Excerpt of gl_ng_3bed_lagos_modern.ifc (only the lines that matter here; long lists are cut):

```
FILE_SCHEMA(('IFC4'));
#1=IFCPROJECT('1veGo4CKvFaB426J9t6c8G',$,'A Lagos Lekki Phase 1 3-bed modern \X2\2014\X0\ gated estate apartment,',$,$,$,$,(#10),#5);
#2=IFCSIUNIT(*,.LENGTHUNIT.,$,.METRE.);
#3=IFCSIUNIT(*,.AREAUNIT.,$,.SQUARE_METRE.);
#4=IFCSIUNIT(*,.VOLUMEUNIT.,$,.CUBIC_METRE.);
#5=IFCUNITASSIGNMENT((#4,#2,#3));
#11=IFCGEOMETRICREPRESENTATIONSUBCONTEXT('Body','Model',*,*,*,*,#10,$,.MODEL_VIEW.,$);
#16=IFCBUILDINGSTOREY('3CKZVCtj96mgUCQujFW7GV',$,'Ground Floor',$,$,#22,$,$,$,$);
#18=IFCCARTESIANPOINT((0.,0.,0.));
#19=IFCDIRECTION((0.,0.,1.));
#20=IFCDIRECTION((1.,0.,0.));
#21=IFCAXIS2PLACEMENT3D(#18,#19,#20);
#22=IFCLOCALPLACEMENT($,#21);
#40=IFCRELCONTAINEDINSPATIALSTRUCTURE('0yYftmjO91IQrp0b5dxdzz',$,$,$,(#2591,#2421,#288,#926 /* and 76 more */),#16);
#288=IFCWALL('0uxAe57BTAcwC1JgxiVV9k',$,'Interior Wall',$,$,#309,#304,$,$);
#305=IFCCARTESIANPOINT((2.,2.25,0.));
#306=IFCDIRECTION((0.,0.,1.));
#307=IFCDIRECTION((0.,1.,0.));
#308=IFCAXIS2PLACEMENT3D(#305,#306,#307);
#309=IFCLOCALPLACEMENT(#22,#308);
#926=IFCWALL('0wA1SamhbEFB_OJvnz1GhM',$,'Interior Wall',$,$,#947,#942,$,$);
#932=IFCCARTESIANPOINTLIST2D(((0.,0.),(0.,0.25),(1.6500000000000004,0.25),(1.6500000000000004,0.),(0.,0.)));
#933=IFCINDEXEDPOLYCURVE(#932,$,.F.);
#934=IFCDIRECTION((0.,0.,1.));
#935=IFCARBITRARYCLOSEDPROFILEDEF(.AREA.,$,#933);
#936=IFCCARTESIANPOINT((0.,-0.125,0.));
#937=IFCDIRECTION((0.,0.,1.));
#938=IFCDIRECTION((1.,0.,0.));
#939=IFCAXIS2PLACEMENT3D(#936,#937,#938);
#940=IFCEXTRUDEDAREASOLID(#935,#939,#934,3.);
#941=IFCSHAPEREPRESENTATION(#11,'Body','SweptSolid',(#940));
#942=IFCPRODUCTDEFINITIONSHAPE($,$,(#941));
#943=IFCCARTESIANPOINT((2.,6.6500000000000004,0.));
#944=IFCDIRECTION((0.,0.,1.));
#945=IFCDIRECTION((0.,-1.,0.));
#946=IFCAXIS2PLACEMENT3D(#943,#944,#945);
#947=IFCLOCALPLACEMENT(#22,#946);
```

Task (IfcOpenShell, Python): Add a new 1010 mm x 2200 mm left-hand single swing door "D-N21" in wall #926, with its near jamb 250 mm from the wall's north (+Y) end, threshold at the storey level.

```python
import numpy as np
import ifcopenshell
import ifcopenshell.api.feature
import ifcopenshell.api.geometry
import ifcopenshell.api.root
import ifcopenshell.api.spatial
import ifcopenshell.geom
import ifcopenshell.util.element
import ifcopenshell.util.placement
import ifcopenshell.util.representation
import ifcopenshell.util.shape
import ifcopenshell.util.unit

model = ifcopenshell.open("gl_ng_3bed_lagos_modern.ifc")
unit_scale = ifcopenshell.util.unit.calculate_unit_scale(model)
settings = ifcopenshell.geom.settings()


def volume(element):
    """Net volume in cubic metres, openings subtracted."""
    shape = ifcopenshell.geom.create_shape(settings, element)
    return ifcopenshell.util.shape.get_volume(shape.geometry)


wall = model.by_guid("0wA1SamhbEFB_OJvnz1GhM")
storey = ifcopenshell.util.element.get_container(wall, ifc_class="IfcBuildingStorey")
context = ifcopenshell.util.representation.get_context(model, "Model", "Body", "MODEL_VIEW")
before = volume(wall)

width, height, from_end, sill = 1.01, 2.2, 0.25, 0.0  # metres

# The wall runs along its own X axis, and the end named is its -X end.
wall_shape = ifcopenshell.geom.create_shape(settings, wall)
x, y, z = ifcopenshell.util.shape.get_vertices(wall_shape.geometry).T
start = x.min() + from_end
face, thickness = float(y.min()), float(y.max() - y.min())
wall_matrix = ifcopenshell.util.placement.get_local_placement(wall.ObjectPlacement)
level = ifcopenshell.util.placement.get_local_placement(storey.ObjectPlacement)[2, 3]


def in_wall(x, y):
    """Placement at x, y metres in the wall's axes, at sill height."""
    matrix = wall_matrix.copy()
    matrix[:, 3] = wall_matrix @ np.array([x / unit_scale, y / unit_scale, 0.0, 1.0])
    matrix[2, 3] = level + sill / unit_scale
    return matrix


# Opening: a box that overshoots both wall faces by 50 mm.
opening = ifcopenshell.api.root.create_entity(model, ifc_class="IfcOpeningElement", predefined_type="OPENING")
box = ifcopenshell.api.geometry.add_wall_representation(
    model, context=context, length=width, height=height, thickness=thickness + 0.1
)
ifcopenshell.api.geometry.assign_representation(model, product=opening, representation=box)
ifcopenshell.api.geometry.edit_object_placement(model, product=opening, matrix=in_wall(start, face - 0.05), is_si=False)
ifcopenshell.api.feature.add_feature(model, feature=opening, element=wall)

door = ifcopenshell.api.root.create_entity(model, ifc_class="IfcDoor", name="D-N21", predefined_type="DOOR")
door.OverallWidth, door.OverallHeight = width / unit_scale, height / unit_scale
door.OperationType = "SINGLE_SWING_LEFT"
body = ifcopenshell.api.geometry.add_door_representation(
    model,
    context=context,
    overall_width=door.OverallWidth,
    overall_height=door.OverallHeight,
    operation_type="SINGLE_SWING_LEFT",
    lining_properties={"LiningDepth": thickness / unit_scale, "ThresholdDepth": thickness / unit_scale},
)
ifcopenshell.api.geometry.assign_representation(model, product=door, representation=body)
ifcopenshell.api.spatial.assign_container(model, products=[door], relating_structure=storey)
ifcopenshell.api.feature.add_filling(model, opening=opening, element=door)

# The lining spans the wall, so the door starts at the wall face.
ifcopenshell.api.geometry.edit_object_placement(model, product=door, matrix=in_wall(start, face), is_si=False)

after = volume(wall)

print(f"wall volume {before:.3f} -> {after:.3f} m3")

model.write("gl_ng_3bed_lagos_modern_updated.ifc")
```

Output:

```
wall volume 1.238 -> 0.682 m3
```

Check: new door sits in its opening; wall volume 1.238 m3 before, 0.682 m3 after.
